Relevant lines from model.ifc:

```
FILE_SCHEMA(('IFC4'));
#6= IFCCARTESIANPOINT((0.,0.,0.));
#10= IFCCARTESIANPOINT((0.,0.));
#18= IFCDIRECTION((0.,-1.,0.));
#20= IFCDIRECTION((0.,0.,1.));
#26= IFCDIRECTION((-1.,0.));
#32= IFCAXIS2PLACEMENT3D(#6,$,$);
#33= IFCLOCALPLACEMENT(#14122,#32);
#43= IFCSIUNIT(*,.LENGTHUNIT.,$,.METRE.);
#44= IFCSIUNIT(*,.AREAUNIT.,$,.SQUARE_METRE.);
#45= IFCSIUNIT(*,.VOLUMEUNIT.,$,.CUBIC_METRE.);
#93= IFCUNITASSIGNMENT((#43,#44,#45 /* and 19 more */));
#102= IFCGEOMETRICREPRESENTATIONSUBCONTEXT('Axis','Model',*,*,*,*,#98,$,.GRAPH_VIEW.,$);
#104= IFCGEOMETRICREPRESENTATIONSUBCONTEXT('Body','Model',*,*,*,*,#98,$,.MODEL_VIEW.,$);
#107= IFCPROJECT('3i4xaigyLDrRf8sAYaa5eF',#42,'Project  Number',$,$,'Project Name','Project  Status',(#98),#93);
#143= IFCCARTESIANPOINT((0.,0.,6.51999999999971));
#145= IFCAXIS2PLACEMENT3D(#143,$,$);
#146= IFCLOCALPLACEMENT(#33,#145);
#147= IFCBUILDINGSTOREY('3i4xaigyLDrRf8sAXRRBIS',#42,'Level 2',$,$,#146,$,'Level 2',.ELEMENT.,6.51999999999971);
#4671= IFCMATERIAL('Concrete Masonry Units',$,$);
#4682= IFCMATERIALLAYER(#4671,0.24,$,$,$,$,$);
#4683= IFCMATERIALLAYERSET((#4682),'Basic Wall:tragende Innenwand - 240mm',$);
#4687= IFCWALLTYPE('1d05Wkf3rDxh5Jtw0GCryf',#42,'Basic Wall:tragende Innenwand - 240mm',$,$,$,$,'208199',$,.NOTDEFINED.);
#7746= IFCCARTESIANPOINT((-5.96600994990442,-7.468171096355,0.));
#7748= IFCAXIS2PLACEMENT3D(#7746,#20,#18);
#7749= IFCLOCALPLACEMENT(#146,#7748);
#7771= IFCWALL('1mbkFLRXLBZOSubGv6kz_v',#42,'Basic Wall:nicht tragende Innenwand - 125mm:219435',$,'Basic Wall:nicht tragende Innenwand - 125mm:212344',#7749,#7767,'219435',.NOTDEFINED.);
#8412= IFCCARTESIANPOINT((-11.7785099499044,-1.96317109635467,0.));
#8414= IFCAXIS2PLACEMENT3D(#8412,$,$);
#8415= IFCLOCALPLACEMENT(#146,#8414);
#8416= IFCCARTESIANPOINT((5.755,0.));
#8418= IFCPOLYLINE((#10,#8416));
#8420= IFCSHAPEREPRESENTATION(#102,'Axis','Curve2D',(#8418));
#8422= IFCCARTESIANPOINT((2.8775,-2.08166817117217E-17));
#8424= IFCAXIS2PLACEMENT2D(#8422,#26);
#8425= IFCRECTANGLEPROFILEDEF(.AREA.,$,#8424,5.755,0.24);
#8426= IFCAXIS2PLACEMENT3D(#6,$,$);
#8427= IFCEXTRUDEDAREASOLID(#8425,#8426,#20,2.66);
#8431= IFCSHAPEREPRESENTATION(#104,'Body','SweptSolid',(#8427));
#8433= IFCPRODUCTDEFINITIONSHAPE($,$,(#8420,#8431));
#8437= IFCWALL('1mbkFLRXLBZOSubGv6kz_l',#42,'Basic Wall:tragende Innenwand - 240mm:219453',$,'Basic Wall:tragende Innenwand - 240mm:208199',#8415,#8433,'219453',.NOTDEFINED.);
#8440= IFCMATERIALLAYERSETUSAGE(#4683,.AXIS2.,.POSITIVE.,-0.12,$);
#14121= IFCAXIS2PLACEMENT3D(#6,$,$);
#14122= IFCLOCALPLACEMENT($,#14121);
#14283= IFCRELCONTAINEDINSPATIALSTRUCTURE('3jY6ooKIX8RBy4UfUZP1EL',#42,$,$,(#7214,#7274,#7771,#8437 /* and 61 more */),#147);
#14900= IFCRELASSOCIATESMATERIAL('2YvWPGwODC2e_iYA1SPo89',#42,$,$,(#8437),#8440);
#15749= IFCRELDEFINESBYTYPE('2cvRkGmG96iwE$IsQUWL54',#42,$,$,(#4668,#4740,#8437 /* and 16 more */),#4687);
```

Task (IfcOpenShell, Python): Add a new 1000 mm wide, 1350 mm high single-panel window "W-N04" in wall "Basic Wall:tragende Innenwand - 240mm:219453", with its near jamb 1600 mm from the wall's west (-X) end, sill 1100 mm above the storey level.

```python
import numpy as np
import ifcopenshell
import ifcopenshell.api.feature
import ifcopenshell.api.geometry
import ifcopenshell.api.root
import ifcopenshell.api.spatial
import ifcopenshell.geom
import ifcopenshell.util.element
import ifcopenshell.util.placement
import ifcopenshell.util.representation
import ifcopenshell.util.shape
import ifcopenshell.util.unit

model = ifcopenshell.open("model.ifc")
unit_scale = ifcopenshell.util.unit.calculate_unit_scale(model)
settings = ifcopenshell.geom.settings()


def volume(element):
    """Net volume in cubic metres, openings subtracted."""
    shape = ifcopenshell.geom.create_shape(settings, element)
    return ifcopenshell.util.shape.get_volume(shape.geometry)


wall = model.by_guid("1mbkFLRXLBZOSubGv6kz_l")
storey = ifcopenshell.util.element.get_container(wall, ifc_class="IfcBuildingStorey")
context = ifcopenshell.util.representation.get_context(model, "Model", "Body", "MODEL_VIEW")
before = volume(wall)

width, height, from_end, sill = 1, 1.35, 1.6, 1.1  # metres

# The wall runs along its own X axis, and the end named is its -X end.
wall_shape = ifcopenshell.geom.create_shape(settings, wall)
x, y, z = ifcopenshell.util.shape.get_vertices(wall_shape.geometry).T
start = x.min() + from_end
face, thickness = float(y.min()), float(y.max() - y.min())
wall_matrix = ifcopenshell.util.placement.get_local_placement(wall.ObjectPlacement)
level = ifcopenshell.util.placement.get_local_placement(storey.ObjectPlacement)[2, 3]


def in_wall(x, y):
    """Placement at x, y metres in the wall's axes, at sill height."""
    matrix = wall_matrix.copy()
    matrix[:, 3] = wall_matrix @ np.array([x / unit_scale, y / unit_scale, 0.0, 1.0])
    matrix[2, 3] = level + sill / unit_scale
    return matrix


# Opening: a box that overshoots both wall faces by 50 mm.
opening = ifcopenshell.api.root.create_entity(model, ifc_class="IfcOpeningElement", predefined_type="OPENING")
box = ifcopenshell.api.geometry.add_wall_representation(
    model, context=context, length=width, height=height, thickness=thickness + 0.1
)
ifcopenshell.api.geometry.assign_representation(model, product=opening, representation=box)
ifcopenshell.api.geometry.edit_object_placement(model, product=opening, matrix=in_wall(start, face - 0.05), is_si=False)
ifcopenshell.api.feature.add_feature(model, feature=opening, element=wall)

window = ifcopenshell.api.root.create_entity(model, ifc_class="IfcWindow", name="W-N04", predefined_type="WINDOW")
window.OverallWidth, window.OverallHeight = width / unit_scale, height / unit_scale
window.PartitioningType = "SINGLE_PANEL"
body = ifcopenshell.api.geometry.add_window_representation(
    model,
    context=context,
    overall_width=window.OverallWidth,
    overall_height=window.OverallHeight,
    partition_type="SINGLE_PANEL",
)
ifcopenshell.api.geometry.assign_representation(model, product=window, representation=body)
ifcopenshell.api.spatial.assign_container(model, products=[window], relating_structure=storey)
ifcopenshell.api.feature.add_filling(model, opening=opening, element=window)

# Centre the window in the wall's thickness.
ifcopenshell.api.geometry.edit_object_placement(model, product=window, matrix=in_wall(start, face), is_si=False)
window_shape = ifcopenshell.geom.create_shape(settings, window)
depth = ifcopenshell.util.shape.get_vertices(window_shape.geometry)[:, 1]
offset = face + thickness / 2 - (depth.min() + depth.max()) / 2
ifcopenshell.api.geometry.edit_object_placement(model, product=window, matrix=in_wall(start, offset), is_si=False)

after = volume(wall)

print(f"wall volume {before:.3f} -> {after:.3f} m3")

model.write("model-out.ifc")
```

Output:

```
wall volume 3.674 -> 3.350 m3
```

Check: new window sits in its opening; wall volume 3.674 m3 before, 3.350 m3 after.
